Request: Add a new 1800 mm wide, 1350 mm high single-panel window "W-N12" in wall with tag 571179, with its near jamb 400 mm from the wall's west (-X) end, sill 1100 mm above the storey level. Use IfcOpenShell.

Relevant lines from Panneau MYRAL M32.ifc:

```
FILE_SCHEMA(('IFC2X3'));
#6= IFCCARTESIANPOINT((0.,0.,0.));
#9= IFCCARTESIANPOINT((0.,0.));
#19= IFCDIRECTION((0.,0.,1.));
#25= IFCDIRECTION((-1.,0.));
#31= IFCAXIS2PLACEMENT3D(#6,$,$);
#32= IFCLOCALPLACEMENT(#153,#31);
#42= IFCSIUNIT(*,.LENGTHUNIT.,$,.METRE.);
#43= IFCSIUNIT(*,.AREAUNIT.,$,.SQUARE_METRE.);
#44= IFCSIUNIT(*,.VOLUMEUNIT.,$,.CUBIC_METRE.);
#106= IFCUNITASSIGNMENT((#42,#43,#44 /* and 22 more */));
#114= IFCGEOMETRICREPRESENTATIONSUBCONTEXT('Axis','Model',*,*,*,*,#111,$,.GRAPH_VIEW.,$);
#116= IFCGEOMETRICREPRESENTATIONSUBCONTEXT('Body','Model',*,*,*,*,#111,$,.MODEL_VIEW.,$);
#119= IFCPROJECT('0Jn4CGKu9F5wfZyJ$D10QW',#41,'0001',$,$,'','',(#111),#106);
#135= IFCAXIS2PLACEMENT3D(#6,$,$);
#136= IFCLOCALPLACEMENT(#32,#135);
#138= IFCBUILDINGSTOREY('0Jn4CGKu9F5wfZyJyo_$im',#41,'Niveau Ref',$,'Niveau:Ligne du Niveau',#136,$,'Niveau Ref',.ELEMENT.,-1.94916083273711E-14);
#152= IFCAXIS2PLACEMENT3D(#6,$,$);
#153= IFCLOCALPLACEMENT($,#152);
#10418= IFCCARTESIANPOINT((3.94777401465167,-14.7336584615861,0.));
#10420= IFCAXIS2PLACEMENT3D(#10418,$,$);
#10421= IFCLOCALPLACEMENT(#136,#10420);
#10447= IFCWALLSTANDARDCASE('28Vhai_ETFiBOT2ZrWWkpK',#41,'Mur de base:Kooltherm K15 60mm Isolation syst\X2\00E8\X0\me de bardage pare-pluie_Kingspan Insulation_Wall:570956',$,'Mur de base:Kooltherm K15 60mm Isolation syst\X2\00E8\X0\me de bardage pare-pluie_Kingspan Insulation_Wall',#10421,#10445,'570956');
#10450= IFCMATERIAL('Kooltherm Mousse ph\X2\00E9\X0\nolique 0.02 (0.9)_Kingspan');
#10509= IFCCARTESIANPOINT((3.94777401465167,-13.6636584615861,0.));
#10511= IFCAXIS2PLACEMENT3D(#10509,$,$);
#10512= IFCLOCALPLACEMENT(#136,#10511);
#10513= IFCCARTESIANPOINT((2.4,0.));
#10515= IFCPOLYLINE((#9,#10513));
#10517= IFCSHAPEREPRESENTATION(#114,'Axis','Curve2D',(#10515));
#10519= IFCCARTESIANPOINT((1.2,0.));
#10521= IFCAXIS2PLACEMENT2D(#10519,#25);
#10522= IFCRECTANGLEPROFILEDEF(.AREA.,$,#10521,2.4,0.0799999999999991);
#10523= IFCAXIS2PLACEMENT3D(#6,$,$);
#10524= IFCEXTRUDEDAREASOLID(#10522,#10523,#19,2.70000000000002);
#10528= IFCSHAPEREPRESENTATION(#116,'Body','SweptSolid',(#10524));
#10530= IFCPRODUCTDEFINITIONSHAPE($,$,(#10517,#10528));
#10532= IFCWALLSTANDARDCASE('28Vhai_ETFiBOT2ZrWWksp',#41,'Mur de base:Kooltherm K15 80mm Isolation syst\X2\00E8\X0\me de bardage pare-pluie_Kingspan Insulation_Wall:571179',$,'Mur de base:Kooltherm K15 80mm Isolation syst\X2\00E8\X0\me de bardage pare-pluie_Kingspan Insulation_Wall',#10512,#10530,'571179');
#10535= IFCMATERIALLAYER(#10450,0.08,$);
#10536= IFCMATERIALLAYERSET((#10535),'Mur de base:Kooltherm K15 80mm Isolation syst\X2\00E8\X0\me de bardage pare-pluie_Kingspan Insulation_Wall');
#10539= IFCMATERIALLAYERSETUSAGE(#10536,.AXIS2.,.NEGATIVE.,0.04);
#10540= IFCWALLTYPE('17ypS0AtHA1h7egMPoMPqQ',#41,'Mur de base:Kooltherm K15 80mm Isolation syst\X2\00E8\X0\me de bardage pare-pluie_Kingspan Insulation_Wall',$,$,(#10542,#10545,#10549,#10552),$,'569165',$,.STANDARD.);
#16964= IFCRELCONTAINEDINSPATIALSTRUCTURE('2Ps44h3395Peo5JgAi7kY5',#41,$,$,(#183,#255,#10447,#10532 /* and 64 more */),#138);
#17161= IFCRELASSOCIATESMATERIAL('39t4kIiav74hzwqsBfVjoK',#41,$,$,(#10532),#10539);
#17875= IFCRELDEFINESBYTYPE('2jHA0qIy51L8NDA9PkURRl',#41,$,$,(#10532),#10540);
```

```python
import numpy as np
import ifcopenshell
import ifcopenshell.api.feature
import ifcopenshell.api.geometry
import ifcopenshell.api.root
import ifcopenshell.api.spatial
import ifcopenshell.api.type
import ifcopenshell.geom
import ifcopenshell.util.element
import ifcopenshell.util.placement
import ifcopenshell.util.representation
import ifcopenshell.util.shape
import ifcopenshell.util.unit

model = ifcopenshell.open("Panneau MYRAL M32.ifc")
unit_scale = ifcopenshell.util.unit.calculate_unit_scale(model)
settings = ifcopenshell.geom.settings()


def volume(element):
    """Net volume in cubic metres, openings subtracted."""
    shape = ifcopenshell.geom.create_shape(settings, element)
    return ifcopenshell.util.shape.get_volume(shape.geometry)


wall = model.by_guid("28Vhai_ETFiBOT2ZrWWksp")
storey = ifcopenshell.util.element.get_container(wall, ifc_class="IfcBuildingStorey")
context = ifcopenshell.util.representation.get_context(model, "Model", "Body", "MODEL_VIEW")
before = volume(wall)

width, height, from_end, sill = 1.8, 1.35, 0.4, 1.1  # metres

# The wall runs along its own X axis, and the end named is its -X end.
wall_shape = ifcopenshell.geom.create_shape(settings, wall)
x, y, z = ifcopenshell.util.shape.get_vertices(wall_shape.geometry).T
start = x.min() + from_end
face, thickness = float(y.min()), float(y.max() - y.min())
wall_matrix = ifcopenshell.util.placement.get_local_placement(wall.ObjectPlacement)
level = ifcopenshell.util.placement.get_local_placement(storey.ObjectPlacement)[2, 3]


def in_wall(x, y):
    """Placement at x, y metres in the wall's axes, at sill height."""
    matrix = wall_matrix.copy()
    matrix[:, 3] = wall_matrix @ np.array([x / unit_scale, y / unit_scale, 0.0, 1.0])
    matrix[2, 3] = level + sill / unit_scale
    return matrix


# Opening: a box that overshoots both wall faces by 50 mm.
opening = ifcopenshell.api.root.create_entity(model, ifc_class="IfcOpeningElement")
box = ifcopenshell.api.geometry.add_wall_representation(
    model, context=context, length=width, height=height, thickness=thickness + 0.1
)
ifcopenshell.api.geometry.assign_representation(model, product=opening, representation=box)
ifcopenshell.api.geometry.edit_object_placement(model, product=opening, matrix=in_wall(start, face - 0.05), is_si=False)
ifcopenshell.api.feature.add_feature(model, feature=opening, element=wall)

window = ifcopenshell.api.root.create_entity(model, ifc_class="IfcWindow", name="W-N12")
window.OverallWidth, window.OverallHeight = width / unit_scale, height / unit_scale
body = ifcopenshell.api.geometry.add_window_representation(
    model,
    context=context,
    overall_width=window.OverallWidth,
    overall_height=window.OverallHeight,
    partition_type="SINGLE_PANEL",
)
ifcopenshell.api.geometry.assign_representation(model, product=window, representation=body)
ifcopenshell.api.spatial.assign_container(model, products=[window], relating_structure=storey)
fills = ifcopenshell.api.feature.add_filling(model, opening=opening, element=window)
fills.OwnerHistory = window.OwnerHistory  # required in IFC2X3

# IFC2X3 keeps the operation on the window style.
style = ifcopenshell.api.root.create_entity(model, ifc_class="IfcWindowStyle", name="W-N12")
style.OperationType, style.ConstructionType = "SINGLE_PANEL", "NOTDEFINED"
style.ParameterTakesPrecedence = style.Sizeable = False
ifcopenshell.api.type.assign_type(model, related_objects=[window], relating_type=style)

# Centre the window in the wall's thickness.
ifcopenshell.api.geometry.edit_object_placement(model, product=window, matrix=in_wall(start, face), is_si=False)
window_shape = ifcopenshell.geom.create_shape(settings, window)
depth = ifcopenshell.util.shape.get_vertices(window_shape.geometry)[:, 1]
offset = face + thickness / 2 - (depth.min() + depth.max()) / 2
ifcopenshell.api.geometry.edit_object_placement(model, product=window, matrix=in_wall(start, offset), is_si=False)

after = volume(wall)

print(f"wall volume {before:.3f} -> {after:.3f} m3")

model.write("Panneau MYRAL M32_updated.ifc")
```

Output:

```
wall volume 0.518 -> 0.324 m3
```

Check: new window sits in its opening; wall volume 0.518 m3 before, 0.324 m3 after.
